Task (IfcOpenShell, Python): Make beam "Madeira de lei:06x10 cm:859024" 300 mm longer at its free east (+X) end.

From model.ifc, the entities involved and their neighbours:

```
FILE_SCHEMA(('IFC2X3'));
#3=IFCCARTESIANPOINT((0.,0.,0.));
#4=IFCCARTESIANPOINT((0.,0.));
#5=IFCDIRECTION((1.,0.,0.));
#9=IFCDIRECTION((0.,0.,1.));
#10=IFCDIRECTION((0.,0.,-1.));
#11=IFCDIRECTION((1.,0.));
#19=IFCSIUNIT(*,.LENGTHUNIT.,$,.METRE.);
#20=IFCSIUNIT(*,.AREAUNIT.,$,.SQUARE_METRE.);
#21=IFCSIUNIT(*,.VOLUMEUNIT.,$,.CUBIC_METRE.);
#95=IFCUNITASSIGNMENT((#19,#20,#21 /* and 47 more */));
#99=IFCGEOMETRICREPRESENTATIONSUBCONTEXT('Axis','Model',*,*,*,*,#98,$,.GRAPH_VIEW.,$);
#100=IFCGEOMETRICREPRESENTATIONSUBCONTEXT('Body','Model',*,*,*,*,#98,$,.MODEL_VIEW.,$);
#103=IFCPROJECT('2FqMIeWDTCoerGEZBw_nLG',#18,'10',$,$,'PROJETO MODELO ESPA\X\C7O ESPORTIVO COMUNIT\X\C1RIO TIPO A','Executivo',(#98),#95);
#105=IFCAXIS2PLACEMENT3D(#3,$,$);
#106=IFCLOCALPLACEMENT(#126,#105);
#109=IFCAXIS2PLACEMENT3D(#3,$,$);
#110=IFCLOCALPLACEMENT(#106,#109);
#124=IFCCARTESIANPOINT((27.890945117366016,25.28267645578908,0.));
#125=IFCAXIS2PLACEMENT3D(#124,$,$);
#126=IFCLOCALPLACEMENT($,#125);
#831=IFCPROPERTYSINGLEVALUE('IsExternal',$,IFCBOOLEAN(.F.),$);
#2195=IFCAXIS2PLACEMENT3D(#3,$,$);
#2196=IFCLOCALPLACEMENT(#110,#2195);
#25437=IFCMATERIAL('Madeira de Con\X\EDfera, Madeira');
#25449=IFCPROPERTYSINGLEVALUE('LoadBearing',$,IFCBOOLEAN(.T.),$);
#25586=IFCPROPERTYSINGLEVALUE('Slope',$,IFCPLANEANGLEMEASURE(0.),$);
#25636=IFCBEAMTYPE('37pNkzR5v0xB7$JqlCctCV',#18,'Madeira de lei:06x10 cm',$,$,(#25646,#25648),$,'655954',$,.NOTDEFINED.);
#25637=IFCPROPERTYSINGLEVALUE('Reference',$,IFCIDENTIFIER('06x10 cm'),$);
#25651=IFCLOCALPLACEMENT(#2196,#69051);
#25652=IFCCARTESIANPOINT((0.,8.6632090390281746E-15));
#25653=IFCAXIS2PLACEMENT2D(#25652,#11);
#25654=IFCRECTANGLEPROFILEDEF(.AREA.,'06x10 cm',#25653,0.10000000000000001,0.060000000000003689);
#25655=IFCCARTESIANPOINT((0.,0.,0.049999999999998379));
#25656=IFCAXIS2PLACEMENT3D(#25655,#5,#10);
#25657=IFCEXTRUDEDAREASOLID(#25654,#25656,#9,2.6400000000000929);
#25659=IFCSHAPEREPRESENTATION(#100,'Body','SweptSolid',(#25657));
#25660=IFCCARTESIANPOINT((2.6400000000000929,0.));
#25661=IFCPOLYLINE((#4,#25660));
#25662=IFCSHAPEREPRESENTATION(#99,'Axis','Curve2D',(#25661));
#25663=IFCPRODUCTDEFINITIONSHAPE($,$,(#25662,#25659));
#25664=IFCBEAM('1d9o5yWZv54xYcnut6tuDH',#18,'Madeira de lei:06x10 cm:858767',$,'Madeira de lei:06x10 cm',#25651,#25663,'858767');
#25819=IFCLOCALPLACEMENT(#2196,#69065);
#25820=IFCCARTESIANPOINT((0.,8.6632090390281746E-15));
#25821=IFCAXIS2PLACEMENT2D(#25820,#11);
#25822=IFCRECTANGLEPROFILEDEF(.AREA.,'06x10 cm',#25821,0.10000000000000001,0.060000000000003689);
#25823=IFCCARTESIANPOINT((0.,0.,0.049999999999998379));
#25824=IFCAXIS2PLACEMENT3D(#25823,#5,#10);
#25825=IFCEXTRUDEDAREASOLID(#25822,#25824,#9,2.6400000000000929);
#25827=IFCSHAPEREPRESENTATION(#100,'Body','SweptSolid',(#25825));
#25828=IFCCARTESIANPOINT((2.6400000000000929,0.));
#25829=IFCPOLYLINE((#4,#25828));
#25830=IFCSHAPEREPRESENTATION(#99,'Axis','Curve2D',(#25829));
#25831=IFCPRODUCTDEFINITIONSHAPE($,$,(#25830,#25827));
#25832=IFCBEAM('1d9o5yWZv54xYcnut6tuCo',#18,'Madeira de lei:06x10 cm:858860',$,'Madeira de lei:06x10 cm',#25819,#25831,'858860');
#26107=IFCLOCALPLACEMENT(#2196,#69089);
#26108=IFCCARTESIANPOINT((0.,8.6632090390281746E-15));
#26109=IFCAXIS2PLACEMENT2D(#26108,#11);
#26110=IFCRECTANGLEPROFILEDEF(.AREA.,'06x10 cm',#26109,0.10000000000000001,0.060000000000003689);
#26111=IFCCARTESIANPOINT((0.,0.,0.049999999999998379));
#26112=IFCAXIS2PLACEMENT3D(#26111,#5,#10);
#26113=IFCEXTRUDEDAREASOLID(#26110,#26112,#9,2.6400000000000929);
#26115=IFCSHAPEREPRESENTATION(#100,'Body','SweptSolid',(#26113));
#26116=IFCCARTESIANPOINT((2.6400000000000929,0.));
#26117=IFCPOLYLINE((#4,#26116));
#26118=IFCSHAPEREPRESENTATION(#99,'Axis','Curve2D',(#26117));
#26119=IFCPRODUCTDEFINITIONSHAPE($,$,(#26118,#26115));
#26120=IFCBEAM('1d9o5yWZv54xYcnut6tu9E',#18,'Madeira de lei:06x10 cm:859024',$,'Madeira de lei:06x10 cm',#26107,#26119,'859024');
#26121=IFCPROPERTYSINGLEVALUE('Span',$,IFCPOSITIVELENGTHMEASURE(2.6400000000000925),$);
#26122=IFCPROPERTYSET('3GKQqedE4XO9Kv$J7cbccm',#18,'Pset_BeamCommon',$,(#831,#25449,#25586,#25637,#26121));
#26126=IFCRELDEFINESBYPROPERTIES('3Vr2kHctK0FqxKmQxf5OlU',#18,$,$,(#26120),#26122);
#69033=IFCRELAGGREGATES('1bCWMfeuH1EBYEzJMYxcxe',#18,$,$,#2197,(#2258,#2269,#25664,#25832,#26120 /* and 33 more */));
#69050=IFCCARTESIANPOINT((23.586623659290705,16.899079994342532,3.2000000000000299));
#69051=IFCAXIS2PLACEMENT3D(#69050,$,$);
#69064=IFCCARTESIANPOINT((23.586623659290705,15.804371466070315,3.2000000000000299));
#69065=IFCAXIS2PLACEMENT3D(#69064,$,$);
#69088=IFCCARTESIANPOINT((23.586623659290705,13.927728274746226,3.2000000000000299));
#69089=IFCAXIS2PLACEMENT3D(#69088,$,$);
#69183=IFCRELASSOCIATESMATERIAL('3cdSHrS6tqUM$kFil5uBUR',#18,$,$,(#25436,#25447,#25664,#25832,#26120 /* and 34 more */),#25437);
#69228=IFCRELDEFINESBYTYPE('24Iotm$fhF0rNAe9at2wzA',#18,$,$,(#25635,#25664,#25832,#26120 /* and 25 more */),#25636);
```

```python
import numpy as np
import ifcopenshell
import ifcopenshell.api.pset
import ifcopenshell.util.element
import ifcopenshell.util.representation
import ifcopenshell.util.unit

model = ifcopenshell.open("model.ifc")
unit_scale = ifcopenshell.util.unit.calculate_unit_scale(model)

member = model.by_id(26120)
change = 0.3 / unit_scale

# The extrusion runs towards the end named, so only its depth changes.
body = ifcopenshell.util.representation.get_representation(member, "Model", "Body")
solid = body.Items[0]
old_length = solid.Depth
solid.Depth += change

# Move the axis end point with it.
axis = next(r for r in member.Representation.Representations if r.RepresentationIdentifier == "Axis").Items[0]
start, end = (np.array(p.Coordinates) for p in axis.Points)
end = end + (end - start) / np.linalg.norm(end - start) * change
point = model.createIfcCartesianPoint(end.tolist())
axis.Points = [axis.Points[0], point]

# Update the stored length and volume.
pset = model.by_id(ifcopenshell.util.element.get_pset(member, "Pset_BeamCommon", should_inherit=False)["id"])
ifcopenshell.api.pset.edit_pset(model, pset=pset, properties={
    "Span": model.create_entity("IfcPositiveLengthMeasure", solid.Depth),
})

print(f"length {old_length:g} -> {solid.Depth:g}")

model.write("model_edited.ifc")
```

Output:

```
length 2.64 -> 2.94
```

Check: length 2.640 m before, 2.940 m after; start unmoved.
